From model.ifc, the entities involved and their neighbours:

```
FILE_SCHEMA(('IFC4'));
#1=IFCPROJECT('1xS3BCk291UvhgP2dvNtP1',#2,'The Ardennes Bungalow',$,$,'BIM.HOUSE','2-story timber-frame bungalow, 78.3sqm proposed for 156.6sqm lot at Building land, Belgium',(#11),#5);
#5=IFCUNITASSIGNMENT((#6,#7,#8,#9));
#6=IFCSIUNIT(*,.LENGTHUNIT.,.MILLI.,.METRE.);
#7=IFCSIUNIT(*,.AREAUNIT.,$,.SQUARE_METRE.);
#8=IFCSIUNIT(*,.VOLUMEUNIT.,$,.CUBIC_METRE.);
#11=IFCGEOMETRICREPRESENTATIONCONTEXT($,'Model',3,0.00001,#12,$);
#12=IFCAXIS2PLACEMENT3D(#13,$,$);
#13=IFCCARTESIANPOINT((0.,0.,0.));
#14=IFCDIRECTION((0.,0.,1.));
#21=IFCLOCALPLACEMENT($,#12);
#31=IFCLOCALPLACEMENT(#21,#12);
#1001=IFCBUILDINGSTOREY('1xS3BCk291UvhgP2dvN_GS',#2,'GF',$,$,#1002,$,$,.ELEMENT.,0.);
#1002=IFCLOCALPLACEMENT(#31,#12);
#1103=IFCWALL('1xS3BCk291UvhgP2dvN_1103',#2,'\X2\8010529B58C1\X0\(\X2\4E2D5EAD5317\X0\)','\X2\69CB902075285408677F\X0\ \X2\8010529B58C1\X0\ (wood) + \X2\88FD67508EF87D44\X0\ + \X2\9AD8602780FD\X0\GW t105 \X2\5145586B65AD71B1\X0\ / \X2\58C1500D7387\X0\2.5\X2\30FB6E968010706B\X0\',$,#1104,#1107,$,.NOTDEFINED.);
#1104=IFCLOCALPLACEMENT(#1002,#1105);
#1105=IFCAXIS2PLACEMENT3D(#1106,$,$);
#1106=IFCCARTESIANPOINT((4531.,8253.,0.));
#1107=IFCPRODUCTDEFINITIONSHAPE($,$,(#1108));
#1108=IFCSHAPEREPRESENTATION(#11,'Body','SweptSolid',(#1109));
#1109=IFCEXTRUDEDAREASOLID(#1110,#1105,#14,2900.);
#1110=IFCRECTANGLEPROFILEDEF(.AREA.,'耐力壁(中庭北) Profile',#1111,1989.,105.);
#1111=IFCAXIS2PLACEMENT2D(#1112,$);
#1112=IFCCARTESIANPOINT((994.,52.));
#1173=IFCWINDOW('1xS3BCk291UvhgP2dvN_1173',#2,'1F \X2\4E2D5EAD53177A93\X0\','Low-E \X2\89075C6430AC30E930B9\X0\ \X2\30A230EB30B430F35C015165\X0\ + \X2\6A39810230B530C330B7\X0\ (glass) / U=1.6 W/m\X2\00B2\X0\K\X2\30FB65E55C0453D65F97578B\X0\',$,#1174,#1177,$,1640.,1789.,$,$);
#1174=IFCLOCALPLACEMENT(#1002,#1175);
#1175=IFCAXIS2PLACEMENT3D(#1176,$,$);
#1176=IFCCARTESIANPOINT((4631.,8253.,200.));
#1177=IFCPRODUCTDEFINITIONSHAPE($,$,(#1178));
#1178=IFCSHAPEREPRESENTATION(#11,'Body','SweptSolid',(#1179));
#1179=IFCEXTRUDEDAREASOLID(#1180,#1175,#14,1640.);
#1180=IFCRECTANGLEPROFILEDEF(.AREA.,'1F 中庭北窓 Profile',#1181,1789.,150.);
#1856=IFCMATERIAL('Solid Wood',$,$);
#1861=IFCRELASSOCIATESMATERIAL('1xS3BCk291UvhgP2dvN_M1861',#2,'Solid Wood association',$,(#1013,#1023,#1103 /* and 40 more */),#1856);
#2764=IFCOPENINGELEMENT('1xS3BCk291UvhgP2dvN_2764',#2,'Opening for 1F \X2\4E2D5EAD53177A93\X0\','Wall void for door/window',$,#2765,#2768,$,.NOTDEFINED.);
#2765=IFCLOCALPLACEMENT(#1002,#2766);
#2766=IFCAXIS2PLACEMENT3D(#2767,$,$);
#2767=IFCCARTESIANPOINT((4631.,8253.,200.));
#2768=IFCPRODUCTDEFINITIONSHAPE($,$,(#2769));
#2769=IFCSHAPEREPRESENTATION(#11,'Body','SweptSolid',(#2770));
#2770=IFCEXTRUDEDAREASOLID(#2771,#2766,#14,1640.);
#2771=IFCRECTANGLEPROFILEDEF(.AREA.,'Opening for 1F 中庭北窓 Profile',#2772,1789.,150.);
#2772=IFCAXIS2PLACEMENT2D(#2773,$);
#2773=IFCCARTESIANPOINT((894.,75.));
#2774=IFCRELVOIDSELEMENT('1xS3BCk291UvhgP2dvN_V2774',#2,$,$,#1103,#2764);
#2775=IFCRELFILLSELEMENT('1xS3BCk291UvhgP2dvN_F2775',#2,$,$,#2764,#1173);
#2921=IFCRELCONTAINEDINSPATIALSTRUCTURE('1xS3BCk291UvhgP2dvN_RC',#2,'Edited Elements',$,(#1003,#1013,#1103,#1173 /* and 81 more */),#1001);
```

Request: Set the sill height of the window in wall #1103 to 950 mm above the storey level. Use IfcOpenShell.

```python
import numpy as np
import ifcopenshell
import ifcopenshell.api.geometry
import ifcopenshell.geom
import ifcopenshell.util.element
import ifcopenshell.util.placement
import ifcopenshell.util.shape
import ifcopenshell.util.unit

model = ifcopenshell.open("model.ifc")
unit_scale = ifcopenshell.util.unit.calculate_unit_scale(model)

window = model.by_guid("1xS3BCk291UvhgP2dvN_1173")
opening = window.FillsVoids[0].RelatingOpeningElement
storey = ifcopenshell.util.element.get_container(window, ifc_class="IfcBuildingStorey")
level = ifcopenshell.util.placement.get_local_placement(storey.ObjectPlacement)[2, 3]

# The opening's origin need not be at the sill, so measure its lowest point.
shape = ifcopenshell.geom.create_shape(ifcopenshell.geom.settings(), opening)
bottom = ifcopenshell.util.shape.get_shape_bottom_elevation(shape, shape.geometry) / unit_scale
dz = level + 0.95 / unit_scale - bottom

shift = np.array([0.0, 0.0, dz])
# The window is not placed relative to its opening, so move both.
for product in (opening, window):
    matrix = ifcopenshell.util.placement.get_local_placement(product.ObjectPlacement)
    matrix[:3, 3] += shift
    ifcopenshell.api.geometry.edit_object_placement(model, product=product, matrix=matrix, is_si=False)

print(f"moved by {dz * unit_scale:+.3f} m")

model.write("model_v2.ifc")
```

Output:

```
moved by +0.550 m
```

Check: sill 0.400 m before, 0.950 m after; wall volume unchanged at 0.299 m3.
